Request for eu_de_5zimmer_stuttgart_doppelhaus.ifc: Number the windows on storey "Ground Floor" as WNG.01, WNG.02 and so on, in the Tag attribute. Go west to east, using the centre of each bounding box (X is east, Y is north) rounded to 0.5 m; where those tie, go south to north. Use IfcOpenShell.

First a look at what the model holds.

```python
import ifcopenshell
import ifcopenshell.util.element
import ifcopenshell.util.placement

model = ifcopenshell.open("eu_de_5zimmer_stuttgart_doppelhaus.ifc")
print(model.schema)
storey = next(s for s in model.by_type("IfcBuildingStorey") if s.Name == "Ground Floor")
windows = [e for e in ifcopenshell.util.element.get_decomposition(storey) if e.is_a("IfcWindow")]
for e in sorted(windows, key=lambda e: e.id()):
    origin = ifcopenshell.util.placement.get_local_placement(e.ObjectPlacement)[:3, 3]
    print(e.id(), e.Tag, e.Name, origin.round(2) + 0.0, sep=" | ")
```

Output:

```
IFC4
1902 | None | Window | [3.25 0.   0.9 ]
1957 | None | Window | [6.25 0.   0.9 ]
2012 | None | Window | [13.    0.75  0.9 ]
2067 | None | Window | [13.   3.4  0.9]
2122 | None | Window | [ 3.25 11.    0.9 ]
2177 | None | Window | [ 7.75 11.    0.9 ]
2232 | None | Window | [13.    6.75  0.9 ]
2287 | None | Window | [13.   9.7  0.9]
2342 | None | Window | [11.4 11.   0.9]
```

```python
import ifcopenshell
import ifcopenshell.geom
import ifcopenshell.util.element
import ifcopenshell.util.shape

model = ifcopenshell.open("eu_de_5zimmer_stuttgart_doppelhaus.ifc")
settings = ifcopenshell.geom.settings()
settings.set("use-world-coords", True)


def centre(element):
    shape = ifcopenshell.geom.create_shape(settings, element)
    return ifcopenshell.util.shape.get_bbox_centroid(shape.geometry)


storey = next(s for s in model.by_type("IfcBuildingStorey") if s.Name == "Ground Floor")
windows = [e for e in ifcopenshell.util.element.get_decomposition(storey) if e.is_a("IfcWindow")]

# Insertion points can sit at a corner or the storey origin, so sort by the geometry (in metres).
centres = {e: centre(e) for e in windows}
windows.sort(key=lambda e: (round(centres[e][0] / 0.5), centres[e][1]))

for i, e in enumerate(windows, start=1):
    number = f"WNG.{i:02d}"
    e.Tag = number
    print(e.id(), number)

model.write("eu_de_5zimmer_stuttgart_doppelhaus-out.ifc")
```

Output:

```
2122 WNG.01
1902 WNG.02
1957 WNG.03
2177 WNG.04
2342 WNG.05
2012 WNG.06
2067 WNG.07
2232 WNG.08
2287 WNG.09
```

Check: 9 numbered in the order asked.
